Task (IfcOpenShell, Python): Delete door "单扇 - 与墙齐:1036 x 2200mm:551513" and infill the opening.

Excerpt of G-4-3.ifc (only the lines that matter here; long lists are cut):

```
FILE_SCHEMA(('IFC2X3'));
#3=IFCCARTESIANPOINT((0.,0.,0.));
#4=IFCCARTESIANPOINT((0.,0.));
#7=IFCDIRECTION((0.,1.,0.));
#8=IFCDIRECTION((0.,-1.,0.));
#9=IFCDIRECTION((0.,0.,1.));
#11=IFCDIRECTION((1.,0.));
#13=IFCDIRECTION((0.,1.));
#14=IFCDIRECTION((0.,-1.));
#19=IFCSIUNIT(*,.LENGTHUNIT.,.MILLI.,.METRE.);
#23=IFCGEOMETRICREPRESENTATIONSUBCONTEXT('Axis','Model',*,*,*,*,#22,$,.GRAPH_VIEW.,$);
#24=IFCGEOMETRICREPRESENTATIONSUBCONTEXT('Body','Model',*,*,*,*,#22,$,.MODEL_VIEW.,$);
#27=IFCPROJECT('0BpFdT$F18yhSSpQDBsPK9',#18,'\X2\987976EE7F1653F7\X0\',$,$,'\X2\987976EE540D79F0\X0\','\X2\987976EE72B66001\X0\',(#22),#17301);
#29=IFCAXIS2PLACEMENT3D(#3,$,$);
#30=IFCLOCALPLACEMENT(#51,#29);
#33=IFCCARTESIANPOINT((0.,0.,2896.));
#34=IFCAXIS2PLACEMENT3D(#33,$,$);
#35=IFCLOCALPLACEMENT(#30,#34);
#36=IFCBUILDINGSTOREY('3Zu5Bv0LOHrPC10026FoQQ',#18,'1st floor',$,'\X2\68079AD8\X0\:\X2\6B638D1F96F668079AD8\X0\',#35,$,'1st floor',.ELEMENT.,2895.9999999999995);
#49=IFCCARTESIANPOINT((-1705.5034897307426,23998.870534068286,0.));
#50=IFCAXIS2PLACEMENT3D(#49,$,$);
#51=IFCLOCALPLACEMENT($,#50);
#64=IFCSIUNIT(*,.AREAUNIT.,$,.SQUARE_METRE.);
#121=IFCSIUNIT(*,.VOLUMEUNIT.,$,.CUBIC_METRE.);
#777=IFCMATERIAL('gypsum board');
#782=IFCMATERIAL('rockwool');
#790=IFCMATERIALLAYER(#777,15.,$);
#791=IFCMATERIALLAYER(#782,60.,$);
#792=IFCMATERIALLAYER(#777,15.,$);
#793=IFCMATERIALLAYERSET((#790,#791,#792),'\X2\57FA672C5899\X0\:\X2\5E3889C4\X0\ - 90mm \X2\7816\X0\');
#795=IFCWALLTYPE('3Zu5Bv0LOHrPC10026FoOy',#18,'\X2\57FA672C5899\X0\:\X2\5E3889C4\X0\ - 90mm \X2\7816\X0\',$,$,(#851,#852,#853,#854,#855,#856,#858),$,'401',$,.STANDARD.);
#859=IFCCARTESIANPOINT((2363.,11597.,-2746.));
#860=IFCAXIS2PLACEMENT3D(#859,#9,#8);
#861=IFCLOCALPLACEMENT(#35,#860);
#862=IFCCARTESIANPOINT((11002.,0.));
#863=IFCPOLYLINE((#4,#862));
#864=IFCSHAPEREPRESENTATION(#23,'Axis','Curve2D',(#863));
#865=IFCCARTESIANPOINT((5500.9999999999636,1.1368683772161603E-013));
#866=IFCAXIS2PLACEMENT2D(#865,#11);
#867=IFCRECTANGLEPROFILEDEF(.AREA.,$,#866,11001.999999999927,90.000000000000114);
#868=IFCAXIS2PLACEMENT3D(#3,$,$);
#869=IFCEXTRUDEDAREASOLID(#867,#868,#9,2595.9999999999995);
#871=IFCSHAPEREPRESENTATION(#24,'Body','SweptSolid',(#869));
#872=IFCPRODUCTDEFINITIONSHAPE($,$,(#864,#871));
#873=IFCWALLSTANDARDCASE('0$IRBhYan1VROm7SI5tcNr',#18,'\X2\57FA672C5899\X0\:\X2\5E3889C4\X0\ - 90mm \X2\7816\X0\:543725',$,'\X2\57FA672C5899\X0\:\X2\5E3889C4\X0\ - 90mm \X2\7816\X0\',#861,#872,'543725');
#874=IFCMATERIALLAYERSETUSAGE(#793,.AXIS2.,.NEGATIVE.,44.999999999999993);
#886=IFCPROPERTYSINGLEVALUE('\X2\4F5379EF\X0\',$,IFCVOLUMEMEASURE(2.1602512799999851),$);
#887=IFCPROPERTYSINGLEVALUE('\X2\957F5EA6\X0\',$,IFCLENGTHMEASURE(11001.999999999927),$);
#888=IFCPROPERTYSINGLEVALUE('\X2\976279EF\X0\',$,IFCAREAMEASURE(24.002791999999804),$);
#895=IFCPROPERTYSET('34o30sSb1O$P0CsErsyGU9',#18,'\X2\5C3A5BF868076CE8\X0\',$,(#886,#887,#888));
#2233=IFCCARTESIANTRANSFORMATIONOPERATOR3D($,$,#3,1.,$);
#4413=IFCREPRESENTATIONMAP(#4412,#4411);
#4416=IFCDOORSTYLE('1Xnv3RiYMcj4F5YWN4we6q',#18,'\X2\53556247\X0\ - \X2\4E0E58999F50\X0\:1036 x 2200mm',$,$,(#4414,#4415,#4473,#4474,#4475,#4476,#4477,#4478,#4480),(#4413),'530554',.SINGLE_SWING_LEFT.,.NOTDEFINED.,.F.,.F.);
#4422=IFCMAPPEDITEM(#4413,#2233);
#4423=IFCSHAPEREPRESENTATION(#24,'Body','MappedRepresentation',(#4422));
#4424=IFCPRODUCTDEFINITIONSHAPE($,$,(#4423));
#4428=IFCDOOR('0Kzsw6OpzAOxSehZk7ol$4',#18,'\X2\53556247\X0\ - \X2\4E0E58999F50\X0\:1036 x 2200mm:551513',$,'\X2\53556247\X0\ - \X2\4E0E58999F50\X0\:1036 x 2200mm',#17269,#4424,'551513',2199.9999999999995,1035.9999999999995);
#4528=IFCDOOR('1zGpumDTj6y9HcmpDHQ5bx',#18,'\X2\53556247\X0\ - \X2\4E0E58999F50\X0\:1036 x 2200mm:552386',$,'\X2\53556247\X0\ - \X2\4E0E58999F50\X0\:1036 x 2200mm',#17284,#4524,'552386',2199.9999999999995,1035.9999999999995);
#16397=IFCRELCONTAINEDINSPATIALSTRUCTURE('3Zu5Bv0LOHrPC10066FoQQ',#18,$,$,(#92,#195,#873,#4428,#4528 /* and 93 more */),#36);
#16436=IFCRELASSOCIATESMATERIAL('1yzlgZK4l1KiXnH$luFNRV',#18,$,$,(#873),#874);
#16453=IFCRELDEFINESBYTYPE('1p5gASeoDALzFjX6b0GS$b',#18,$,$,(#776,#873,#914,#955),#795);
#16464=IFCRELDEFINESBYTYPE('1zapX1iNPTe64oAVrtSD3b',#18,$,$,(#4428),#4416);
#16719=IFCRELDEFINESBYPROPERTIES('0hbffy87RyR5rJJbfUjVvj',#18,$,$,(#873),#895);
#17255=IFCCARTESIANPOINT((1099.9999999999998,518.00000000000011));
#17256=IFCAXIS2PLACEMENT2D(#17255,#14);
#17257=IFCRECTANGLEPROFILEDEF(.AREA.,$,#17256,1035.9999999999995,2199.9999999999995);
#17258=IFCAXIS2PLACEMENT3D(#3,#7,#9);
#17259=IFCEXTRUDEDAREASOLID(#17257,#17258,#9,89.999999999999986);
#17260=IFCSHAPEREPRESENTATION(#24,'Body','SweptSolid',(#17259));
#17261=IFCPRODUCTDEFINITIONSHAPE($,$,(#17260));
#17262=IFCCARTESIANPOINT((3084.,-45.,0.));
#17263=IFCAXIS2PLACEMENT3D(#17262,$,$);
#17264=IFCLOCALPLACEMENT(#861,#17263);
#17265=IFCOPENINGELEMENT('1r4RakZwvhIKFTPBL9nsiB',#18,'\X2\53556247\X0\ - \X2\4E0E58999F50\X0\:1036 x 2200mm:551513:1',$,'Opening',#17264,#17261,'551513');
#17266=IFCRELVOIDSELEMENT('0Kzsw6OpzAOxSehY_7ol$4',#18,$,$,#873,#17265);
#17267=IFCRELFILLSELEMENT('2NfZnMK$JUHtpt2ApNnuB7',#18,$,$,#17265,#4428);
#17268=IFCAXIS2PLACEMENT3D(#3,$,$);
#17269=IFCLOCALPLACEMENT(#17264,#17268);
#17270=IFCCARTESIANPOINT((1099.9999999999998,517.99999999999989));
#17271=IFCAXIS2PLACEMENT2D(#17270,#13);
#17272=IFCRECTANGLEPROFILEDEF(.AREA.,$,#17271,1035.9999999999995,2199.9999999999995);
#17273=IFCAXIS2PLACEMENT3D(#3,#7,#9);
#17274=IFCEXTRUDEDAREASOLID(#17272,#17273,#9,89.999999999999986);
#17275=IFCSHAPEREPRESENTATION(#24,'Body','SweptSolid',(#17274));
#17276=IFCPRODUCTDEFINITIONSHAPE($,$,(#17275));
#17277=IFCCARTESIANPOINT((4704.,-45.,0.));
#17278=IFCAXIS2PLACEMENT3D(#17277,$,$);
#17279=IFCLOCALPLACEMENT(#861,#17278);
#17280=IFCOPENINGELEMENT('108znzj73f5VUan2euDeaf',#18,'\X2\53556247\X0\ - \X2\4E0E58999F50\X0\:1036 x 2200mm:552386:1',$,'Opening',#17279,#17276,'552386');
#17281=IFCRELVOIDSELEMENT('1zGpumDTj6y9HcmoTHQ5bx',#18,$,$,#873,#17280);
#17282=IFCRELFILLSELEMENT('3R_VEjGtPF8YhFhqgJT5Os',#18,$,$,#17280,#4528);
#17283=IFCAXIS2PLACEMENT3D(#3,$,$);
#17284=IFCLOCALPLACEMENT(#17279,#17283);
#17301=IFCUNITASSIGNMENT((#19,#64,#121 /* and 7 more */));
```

```python
import ifcopenshell
import ifcopenshell.api.feature
import ifcopenshell.api.pset
import ifcopenshell.api.root
import ifcopenshell.geom
import ifcopenshell.util.element
import ifcopenshell.util.shape
import ifcopenshell.util.unit

model = ifcopenshell.open("G-4-3.ifc")
area_scale = ifcopenshell.util.unit.calculate_unit_scale(model, "AREAUNIT")
volume_scale = ifcopenshell.util.unit.calculate_unit_scale(model, "VOLUMEUNIT")
settings = ifcopenshell.geom.settings()


def volume(element):
    """Net volume in cubic metres, openings subtracted."""
    shape = ifcopenshell.geom.create_shape(settings, element)
    return ifcopenshell.util.shape.get_volume(shape.geometry)


door = model.by_guid("0Kzsw6OpzAOxSehZk7ol$4")
opening = door.FillsVoids[0].RelatingOpeningElement
wall = opening.VoidsElements[0].RelatingBuildingElement
before = volume(wall)

ifcopenshell.api.root.remove_product(model, product=door)
ifcopenshell.api.feature.remove_feature(model, feature=opening)

after = volume(wall)
thickness = 0.09  # wall thickness in metres

# Update the wall's stored quantities.
pset = model.by_id(ifcopenshell.util.element.get_pset(wall, "尺寸标注", should_inherit=False)["id"])
ifcopenshell.api.pset.edit_pset(model, pset=pset, properties={
    "体积": model.create_entity("IfcVolumeMeasure", after / volume_scale),
    "面积": model.create_entity("IfcAreaMeasure", after / thickness / area_scale),
})

print(f"wall volume {before:.3f} -> {after:.3f} m3")

model.write("G-4-3_rev.ifc")
```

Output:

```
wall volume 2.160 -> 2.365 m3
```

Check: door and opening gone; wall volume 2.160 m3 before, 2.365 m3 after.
